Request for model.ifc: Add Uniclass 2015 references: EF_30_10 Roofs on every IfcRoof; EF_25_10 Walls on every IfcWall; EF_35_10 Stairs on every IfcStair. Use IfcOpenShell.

First a look at what the model holds.

```python
import ifcopenshell

model = ifcopenshell.open("model.ifc")
print(model.schema)
print("classifications:", [c.Name for c in model.by_type("IfcClassification")])
for ifc_class in ("IfcDoor", "IfcRoof", "IfcStair", "IfcWall", "IfcWindow"):
    print(ifc_class, len(model.by_type(ifc_class)))
```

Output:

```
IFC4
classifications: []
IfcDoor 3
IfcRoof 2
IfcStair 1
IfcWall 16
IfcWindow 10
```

```python
import ifcopenshell
import ifcopenshell.api.classification

model = ifcopenshell.open("model.ifc")

system = ifcopenshell.api.classification.add_classification(model, classification="Uniclass 2015")

codes = {
    "IfcRoof": ("EF_30_10", "Roofs"),
    "IfcWall": ("EF_25_10", "Walls"),
    "IfcStair": ("EF_35_10", "Stairs"),
}
for ifc_class, (code, name) in codes.items():
    products = model.by_type(ifc_class)
    ifcopenshell.api.classification.add_reference(
        model, products=products, classification=system, identification=code, name=name
    )
    print(code, len(products))

model.write("model-out.ifc")
```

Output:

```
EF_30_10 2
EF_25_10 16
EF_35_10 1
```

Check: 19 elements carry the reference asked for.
